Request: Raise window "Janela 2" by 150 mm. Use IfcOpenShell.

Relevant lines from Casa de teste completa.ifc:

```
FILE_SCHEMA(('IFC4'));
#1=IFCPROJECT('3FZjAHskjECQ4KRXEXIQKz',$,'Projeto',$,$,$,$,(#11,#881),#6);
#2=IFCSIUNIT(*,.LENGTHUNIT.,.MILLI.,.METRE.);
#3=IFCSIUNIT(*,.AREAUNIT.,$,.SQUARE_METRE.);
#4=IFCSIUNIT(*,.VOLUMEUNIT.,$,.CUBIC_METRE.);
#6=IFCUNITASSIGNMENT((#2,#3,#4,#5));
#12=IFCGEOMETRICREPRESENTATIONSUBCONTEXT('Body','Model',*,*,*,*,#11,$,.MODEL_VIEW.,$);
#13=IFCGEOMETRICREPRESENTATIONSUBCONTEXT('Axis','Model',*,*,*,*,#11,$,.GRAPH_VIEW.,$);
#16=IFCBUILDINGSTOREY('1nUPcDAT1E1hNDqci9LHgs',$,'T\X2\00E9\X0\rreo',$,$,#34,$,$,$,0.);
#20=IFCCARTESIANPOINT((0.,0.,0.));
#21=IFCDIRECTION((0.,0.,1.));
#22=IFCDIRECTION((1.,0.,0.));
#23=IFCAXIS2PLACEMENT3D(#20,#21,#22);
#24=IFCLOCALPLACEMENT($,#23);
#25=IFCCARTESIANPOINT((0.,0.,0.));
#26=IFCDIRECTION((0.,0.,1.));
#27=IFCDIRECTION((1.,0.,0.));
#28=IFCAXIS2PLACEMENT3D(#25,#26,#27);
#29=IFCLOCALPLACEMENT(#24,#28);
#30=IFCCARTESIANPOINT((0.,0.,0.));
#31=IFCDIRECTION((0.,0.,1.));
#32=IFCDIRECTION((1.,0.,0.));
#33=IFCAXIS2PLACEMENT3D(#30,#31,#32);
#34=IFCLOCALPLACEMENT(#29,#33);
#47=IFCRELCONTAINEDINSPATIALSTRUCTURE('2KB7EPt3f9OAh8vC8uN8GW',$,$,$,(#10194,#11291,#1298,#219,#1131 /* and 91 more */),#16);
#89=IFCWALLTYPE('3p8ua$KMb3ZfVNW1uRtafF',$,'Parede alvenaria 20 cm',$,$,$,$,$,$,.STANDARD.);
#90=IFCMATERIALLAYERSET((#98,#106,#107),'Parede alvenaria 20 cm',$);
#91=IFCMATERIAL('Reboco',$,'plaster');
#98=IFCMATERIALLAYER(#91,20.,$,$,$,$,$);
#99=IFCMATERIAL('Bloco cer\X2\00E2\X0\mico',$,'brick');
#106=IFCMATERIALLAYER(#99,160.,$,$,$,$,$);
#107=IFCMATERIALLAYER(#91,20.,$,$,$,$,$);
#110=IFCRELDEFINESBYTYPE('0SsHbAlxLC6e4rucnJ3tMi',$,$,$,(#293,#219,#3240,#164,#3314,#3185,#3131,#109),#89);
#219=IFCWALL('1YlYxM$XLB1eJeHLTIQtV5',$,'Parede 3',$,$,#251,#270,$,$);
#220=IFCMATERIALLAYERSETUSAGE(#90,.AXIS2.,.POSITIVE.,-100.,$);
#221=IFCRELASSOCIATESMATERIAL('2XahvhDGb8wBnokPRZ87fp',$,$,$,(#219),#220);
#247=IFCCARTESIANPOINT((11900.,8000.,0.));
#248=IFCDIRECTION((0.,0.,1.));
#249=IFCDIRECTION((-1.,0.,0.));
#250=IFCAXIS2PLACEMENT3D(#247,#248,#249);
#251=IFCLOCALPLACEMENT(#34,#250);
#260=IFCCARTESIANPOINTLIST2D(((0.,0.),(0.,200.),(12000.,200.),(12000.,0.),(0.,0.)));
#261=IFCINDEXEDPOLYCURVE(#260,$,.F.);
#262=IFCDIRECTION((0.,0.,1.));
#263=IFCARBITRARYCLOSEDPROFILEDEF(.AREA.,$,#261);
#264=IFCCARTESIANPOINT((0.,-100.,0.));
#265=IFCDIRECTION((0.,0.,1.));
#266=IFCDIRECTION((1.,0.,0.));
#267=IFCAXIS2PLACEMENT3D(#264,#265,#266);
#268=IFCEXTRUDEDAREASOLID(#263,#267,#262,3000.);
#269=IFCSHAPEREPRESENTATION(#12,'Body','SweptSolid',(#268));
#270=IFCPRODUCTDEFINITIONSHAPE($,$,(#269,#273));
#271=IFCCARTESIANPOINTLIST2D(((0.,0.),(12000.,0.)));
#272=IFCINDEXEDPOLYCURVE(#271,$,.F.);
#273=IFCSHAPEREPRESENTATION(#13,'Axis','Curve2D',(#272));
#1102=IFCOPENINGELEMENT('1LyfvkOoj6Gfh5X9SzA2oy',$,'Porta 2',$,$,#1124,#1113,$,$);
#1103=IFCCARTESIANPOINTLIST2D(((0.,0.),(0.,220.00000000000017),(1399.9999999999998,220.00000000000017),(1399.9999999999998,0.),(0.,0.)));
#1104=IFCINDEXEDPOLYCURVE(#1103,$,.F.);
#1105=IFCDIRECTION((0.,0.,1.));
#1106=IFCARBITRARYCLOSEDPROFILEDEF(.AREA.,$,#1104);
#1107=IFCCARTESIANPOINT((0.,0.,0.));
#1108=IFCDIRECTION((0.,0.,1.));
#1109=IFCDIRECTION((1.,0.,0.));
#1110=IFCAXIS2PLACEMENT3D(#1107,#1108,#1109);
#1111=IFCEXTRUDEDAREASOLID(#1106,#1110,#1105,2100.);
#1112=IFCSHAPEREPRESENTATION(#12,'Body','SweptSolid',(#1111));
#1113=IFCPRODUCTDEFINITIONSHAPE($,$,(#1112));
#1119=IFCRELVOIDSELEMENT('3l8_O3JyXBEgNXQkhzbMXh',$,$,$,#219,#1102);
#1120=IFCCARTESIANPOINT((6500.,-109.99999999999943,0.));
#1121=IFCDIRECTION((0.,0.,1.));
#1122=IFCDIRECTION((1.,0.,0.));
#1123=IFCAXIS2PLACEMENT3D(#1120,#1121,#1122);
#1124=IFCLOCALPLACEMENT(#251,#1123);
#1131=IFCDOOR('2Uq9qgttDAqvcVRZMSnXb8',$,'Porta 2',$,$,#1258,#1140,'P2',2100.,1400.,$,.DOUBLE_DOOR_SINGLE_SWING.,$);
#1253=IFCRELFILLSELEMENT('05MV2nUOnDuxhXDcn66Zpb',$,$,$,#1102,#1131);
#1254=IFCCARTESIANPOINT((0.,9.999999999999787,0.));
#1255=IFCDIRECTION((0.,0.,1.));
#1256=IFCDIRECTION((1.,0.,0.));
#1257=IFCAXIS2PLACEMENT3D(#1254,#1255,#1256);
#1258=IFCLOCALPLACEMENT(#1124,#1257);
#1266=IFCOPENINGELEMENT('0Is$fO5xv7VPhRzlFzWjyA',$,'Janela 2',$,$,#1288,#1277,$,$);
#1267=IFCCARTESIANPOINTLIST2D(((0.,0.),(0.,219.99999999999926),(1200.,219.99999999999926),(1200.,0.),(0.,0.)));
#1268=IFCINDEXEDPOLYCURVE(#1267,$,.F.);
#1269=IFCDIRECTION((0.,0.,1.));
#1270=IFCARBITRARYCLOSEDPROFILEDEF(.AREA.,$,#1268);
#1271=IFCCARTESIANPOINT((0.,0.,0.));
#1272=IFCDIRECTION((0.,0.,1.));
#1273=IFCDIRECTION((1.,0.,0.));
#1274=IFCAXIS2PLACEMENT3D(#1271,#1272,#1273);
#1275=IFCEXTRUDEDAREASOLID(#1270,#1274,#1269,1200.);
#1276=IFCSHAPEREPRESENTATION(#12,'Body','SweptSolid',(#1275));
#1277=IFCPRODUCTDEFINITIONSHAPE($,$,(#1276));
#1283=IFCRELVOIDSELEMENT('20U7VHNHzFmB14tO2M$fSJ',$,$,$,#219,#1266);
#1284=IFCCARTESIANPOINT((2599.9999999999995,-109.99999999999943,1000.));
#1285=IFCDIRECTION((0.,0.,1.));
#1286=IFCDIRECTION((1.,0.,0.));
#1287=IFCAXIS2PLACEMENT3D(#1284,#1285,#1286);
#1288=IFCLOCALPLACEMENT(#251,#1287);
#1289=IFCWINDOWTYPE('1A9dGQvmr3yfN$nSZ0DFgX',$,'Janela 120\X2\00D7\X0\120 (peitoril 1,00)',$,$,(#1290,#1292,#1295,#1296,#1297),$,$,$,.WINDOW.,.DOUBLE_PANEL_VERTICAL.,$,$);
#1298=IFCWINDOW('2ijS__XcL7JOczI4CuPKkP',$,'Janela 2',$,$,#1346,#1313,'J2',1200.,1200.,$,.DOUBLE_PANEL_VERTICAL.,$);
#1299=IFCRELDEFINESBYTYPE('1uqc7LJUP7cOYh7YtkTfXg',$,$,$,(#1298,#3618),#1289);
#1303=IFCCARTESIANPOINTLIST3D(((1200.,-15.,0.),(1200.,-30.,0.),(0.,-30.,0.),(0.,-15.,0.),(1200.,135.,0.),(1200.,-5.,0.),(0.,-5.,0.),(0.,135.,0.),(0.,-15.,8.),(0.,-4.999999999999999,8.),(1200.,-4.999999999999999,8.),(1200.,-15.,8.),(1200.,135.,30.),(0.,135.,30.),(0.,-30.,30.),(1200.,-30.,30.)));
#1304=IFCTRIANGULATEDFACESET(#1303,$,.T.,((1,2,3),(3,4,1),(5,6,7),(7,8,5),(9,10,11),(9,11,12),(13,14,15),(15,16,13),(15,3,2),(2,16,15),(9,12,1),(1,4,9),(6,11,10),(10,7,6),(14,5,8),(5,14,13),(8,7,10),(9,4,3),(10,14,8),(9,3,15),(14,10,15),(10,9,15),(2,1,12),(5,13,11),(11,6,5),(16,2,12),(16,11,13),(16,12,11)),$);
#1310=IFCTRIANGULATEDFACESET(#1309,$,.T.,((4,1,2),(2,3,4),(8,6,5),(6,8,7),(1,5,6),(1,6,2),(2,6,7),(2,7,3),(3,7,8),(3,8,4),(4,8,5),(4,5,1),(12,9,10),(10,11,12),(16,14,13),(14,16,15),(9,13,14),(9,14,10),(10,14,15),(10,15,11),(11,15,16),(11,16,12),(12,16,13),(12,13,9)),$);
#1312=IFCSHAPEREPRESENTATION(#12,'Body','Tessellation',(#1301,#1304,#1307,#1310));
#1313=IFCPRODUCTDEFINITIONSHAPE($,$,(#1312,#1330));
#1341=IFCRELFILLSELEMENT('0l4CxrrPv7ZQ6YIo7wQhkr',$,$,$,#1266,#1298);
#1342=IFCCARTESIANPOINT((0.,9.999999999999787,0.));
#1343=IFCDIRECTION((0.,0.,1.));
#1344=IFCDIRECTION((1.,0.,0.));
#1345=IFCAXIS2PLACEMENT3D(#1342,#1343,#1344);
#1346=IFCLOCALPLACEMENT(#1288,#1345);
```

```python
import numpy as np
import ifcopenshell
import ifcopenshell.api.geometry
import ifcopenshell.util.placement
import ifcopenshell.util.unit

model = ifcopenshell.open("Casa de teste completa.ifc")
unit_scale = ifcopenshell.util.unit.calculate_unit_scale(model)

window = model.by_id(1298)
opening = window.FillsVoids[0].RelatingOpeningElement
dz = 0.15 / unit_scale

shift = np.array([0.0, 0.0, dz])
# The window is placed relative to its opening, so it follows when the opening moves.
matrix = ifcopenshell.util.placement.get_local_placement(opening.ObjectPlacement)
matrix[:3, 3] += shift
ifcopenshell.api.geometry.edit_object_placement(
    model, product=opening, matrix=matrix, is_si=False, should_transform_children=True
)

print(f"moved by {dz * unit_scale:+.3f} m")

model.write("Casa de teste completa_rev.ifc")
```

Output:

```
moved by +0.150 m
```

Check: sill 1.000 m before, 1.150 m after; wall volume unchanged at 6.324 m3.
